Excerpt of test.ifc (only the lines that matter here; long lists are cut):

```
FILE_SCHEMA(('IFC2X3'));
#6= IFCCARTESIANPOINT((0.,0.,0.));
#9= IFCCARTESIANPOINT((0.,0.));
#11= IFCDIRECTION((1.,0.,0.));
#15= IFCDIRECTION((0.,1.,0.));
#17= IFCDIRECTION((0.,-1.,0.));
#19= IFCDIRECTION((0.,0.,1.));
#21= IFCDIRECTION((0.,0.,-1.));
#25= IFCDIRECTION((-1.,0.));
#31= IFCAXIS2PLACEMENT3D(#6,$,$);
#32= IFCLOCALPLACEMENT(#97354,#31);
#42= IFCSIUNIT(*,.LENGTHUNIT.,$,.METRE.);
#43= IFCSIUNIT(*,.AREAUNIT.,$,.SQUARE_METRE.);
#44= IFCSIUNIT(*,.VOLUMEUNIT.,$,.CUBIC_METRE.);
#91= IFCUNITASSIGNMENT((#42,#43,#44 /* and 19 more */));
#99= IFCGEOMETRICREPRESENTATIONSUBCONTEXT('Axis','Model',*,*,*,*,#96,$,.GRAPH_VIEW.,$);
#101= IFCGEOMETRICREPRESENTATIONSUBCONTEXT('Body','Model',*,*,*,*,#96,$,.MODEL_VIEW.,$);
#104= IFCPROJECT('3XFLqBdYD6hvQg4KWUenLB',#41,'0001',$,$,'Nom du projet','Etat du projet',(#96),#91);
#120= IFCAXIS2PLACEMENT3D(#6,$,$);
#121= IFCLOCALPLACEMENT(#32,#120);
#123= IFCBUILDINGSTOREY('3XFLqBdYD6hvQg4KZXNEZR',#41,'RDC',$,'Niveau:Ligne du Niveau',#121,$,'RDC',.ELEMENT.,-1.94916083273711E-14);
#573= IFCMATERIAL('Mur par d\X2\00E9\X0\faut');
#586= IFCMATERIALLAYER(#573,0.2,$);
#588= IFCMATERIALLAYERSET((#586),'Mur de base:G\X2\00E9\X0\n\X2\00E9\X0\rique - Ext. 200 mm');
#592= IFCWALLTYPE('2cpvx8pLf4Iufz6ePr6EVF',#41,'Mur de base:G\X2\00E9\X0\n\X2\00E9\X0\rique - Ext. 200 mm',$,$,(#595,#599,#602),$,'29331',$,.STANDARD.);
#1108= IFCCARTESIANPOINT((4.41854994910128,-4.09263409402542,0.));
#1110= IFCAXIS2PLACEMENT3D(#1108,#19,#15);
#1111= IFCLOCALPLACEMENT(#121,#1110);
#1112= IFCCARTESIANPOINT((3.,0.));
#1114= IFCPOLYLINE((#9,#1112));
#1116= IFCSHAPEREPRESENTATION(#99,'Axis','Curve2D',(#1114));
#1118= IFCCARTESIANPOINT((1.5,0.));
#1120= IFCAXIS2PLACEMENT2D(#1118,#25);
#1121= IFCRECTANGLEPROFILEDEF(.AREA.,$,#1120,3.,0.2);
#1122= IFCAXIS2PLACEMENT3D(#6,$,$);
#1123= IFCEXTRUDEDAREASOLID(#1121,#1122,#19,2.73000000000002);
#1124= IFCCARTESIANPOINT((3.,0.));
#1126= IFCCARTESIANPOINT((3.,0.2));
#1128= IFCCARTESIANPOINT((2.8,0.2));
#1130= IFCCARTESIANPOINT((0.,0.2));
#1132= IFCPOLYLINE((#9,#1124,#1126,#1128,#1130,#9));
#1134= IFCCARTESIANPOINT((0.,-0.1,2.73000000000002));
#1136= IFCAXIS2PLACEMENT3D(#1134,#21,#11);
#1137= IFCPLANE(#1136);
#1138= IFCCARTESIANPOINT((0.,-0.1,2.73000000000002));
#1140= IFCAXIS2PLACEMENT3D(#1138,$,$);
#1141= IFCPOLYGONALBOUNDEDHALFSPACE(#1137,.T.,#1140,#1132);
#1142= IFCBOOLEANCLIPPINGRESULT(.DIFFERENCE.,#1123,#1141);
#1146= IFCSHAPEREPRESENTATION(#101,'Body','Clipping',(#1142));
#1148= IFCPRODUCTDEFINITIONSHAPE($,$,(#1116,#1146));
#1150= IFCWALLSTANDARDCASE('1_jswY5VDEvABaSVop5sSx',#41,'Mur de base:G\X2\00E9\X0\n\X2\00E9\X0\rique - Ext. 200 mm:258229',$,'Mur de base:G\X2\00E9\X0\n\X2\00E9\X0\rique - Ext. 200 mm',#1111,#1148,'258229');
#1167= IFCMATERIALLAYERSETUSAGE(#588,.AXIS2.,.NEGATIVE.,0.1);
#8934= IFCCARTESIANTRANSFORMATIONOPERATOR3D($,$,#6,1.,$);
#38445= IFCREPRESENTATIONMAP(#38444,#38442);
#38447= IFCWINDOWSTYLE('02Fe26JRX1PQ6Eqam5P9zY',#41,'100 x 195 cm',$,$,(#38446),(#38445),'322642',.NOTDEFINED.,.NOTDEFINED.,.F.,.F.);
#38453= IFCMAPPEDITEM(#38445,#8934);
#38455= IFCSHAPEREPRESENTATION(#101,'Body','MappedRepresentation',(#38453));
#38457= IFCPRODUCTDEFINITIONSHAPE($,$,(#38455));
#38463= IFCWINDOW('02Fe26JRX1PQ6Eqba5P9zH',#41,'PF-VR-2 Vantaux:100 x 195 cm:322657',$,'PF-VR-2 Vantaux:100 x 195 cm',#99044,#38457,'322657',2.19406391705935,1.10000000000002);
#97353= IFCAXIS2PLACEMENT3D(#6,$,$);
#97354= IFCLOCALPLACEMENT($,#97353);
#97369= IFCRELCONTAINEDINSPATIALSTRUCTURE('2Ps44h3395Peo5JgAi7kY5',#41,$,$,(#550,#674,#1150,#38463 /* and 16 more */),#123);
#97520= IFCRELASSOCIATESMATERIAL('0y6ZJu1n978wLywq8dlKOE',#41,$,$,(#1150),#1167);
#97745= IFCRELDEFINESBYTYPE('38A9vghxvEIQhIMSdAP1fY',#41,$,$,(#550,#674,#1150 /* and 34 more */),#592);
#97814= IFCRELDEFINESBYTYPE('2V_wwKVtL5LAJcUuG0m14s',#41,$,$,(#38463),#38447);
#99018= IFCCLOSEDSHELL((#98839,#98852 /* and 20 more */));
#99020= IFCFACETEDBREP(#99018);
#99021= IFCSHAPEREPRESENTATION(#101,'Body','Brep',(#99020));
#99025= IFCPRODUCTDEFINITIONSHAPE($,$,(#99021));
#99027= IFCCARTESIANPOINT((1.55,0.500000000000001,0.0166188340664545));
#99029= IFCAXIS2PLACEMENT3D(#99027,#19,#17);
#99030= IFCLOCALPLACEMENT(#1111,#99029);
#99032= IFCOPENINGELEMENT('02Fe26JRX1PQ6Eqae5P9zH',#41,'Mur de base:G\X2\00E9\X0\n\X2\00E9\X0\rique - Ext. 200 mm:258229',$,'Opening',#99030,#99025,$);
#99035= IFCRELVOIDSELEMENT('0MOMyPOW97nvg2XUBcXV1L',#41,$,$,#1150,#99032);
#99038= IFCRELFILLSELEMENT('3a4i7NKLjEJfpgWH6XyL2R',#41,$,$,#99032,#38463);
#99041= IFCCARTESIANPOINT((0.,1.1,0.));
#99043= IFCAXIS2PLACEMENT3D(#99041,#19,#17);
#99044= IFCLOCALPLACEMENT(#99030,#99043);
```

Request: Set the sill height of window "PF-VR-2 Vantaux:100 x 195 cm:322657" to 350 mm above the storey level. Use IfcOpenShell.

```python
import numpy as np
import ifcopenshell
import ifcopenshell.api.geometry
import ifcopenshell.geom
import ifcopenshell.util.element
import ifcopenshell.util.placement
import ifcopenshell.util.shape
import ifcopenshell.util.unit

model = ifcopenshell.open("test.ifc")
unit_scale = ifcopenshell.util.unit.calculate_unit_scale(model)

window = model.by_guid("02Fe26JRX1PQ6Eqba5P9zH")
opening = window.FillsVoids[0].RelatingOpeningElement
storey = ifcopenshell.util.element.get_container(window, ifc_class="IfcBuildingStorey")
level = ifcopenshell.util.placement.get_local_placement(storey.ObjectPlacement)[2, 3]

# The opening's origin need not be at the sill, so measure its lowest point.
shape = ifcopenshell.geom.create_shape(ifcopenshell.geom.settings(), opening)
bottom = ifcopenshell.util.shape.get_shape_bottom_elevation(shape, shape.geometry) / unit_scale
dz = level + 0.35 - bottom

shift = np.array([0.0, 0.0, dz])
# The window is placed relative to its opening, so it follows when the opening moves.
matrix = ifcopenshell.util.placement.get_local_placement(opening.ObjectPlacement)
matrix[:3, 3] += shift
ifcopenshell.api.geometry.edit_object_placement(
    model, product=opening, matrix=matrix, is_si=False, should_transform_children=True
)

print(f"moved by {dz * unit_scale:+.3f} m")

model.write("test_v2.ifc")
```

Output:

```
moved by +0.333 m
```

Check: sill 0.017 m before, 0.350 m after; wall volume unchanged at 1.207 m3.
